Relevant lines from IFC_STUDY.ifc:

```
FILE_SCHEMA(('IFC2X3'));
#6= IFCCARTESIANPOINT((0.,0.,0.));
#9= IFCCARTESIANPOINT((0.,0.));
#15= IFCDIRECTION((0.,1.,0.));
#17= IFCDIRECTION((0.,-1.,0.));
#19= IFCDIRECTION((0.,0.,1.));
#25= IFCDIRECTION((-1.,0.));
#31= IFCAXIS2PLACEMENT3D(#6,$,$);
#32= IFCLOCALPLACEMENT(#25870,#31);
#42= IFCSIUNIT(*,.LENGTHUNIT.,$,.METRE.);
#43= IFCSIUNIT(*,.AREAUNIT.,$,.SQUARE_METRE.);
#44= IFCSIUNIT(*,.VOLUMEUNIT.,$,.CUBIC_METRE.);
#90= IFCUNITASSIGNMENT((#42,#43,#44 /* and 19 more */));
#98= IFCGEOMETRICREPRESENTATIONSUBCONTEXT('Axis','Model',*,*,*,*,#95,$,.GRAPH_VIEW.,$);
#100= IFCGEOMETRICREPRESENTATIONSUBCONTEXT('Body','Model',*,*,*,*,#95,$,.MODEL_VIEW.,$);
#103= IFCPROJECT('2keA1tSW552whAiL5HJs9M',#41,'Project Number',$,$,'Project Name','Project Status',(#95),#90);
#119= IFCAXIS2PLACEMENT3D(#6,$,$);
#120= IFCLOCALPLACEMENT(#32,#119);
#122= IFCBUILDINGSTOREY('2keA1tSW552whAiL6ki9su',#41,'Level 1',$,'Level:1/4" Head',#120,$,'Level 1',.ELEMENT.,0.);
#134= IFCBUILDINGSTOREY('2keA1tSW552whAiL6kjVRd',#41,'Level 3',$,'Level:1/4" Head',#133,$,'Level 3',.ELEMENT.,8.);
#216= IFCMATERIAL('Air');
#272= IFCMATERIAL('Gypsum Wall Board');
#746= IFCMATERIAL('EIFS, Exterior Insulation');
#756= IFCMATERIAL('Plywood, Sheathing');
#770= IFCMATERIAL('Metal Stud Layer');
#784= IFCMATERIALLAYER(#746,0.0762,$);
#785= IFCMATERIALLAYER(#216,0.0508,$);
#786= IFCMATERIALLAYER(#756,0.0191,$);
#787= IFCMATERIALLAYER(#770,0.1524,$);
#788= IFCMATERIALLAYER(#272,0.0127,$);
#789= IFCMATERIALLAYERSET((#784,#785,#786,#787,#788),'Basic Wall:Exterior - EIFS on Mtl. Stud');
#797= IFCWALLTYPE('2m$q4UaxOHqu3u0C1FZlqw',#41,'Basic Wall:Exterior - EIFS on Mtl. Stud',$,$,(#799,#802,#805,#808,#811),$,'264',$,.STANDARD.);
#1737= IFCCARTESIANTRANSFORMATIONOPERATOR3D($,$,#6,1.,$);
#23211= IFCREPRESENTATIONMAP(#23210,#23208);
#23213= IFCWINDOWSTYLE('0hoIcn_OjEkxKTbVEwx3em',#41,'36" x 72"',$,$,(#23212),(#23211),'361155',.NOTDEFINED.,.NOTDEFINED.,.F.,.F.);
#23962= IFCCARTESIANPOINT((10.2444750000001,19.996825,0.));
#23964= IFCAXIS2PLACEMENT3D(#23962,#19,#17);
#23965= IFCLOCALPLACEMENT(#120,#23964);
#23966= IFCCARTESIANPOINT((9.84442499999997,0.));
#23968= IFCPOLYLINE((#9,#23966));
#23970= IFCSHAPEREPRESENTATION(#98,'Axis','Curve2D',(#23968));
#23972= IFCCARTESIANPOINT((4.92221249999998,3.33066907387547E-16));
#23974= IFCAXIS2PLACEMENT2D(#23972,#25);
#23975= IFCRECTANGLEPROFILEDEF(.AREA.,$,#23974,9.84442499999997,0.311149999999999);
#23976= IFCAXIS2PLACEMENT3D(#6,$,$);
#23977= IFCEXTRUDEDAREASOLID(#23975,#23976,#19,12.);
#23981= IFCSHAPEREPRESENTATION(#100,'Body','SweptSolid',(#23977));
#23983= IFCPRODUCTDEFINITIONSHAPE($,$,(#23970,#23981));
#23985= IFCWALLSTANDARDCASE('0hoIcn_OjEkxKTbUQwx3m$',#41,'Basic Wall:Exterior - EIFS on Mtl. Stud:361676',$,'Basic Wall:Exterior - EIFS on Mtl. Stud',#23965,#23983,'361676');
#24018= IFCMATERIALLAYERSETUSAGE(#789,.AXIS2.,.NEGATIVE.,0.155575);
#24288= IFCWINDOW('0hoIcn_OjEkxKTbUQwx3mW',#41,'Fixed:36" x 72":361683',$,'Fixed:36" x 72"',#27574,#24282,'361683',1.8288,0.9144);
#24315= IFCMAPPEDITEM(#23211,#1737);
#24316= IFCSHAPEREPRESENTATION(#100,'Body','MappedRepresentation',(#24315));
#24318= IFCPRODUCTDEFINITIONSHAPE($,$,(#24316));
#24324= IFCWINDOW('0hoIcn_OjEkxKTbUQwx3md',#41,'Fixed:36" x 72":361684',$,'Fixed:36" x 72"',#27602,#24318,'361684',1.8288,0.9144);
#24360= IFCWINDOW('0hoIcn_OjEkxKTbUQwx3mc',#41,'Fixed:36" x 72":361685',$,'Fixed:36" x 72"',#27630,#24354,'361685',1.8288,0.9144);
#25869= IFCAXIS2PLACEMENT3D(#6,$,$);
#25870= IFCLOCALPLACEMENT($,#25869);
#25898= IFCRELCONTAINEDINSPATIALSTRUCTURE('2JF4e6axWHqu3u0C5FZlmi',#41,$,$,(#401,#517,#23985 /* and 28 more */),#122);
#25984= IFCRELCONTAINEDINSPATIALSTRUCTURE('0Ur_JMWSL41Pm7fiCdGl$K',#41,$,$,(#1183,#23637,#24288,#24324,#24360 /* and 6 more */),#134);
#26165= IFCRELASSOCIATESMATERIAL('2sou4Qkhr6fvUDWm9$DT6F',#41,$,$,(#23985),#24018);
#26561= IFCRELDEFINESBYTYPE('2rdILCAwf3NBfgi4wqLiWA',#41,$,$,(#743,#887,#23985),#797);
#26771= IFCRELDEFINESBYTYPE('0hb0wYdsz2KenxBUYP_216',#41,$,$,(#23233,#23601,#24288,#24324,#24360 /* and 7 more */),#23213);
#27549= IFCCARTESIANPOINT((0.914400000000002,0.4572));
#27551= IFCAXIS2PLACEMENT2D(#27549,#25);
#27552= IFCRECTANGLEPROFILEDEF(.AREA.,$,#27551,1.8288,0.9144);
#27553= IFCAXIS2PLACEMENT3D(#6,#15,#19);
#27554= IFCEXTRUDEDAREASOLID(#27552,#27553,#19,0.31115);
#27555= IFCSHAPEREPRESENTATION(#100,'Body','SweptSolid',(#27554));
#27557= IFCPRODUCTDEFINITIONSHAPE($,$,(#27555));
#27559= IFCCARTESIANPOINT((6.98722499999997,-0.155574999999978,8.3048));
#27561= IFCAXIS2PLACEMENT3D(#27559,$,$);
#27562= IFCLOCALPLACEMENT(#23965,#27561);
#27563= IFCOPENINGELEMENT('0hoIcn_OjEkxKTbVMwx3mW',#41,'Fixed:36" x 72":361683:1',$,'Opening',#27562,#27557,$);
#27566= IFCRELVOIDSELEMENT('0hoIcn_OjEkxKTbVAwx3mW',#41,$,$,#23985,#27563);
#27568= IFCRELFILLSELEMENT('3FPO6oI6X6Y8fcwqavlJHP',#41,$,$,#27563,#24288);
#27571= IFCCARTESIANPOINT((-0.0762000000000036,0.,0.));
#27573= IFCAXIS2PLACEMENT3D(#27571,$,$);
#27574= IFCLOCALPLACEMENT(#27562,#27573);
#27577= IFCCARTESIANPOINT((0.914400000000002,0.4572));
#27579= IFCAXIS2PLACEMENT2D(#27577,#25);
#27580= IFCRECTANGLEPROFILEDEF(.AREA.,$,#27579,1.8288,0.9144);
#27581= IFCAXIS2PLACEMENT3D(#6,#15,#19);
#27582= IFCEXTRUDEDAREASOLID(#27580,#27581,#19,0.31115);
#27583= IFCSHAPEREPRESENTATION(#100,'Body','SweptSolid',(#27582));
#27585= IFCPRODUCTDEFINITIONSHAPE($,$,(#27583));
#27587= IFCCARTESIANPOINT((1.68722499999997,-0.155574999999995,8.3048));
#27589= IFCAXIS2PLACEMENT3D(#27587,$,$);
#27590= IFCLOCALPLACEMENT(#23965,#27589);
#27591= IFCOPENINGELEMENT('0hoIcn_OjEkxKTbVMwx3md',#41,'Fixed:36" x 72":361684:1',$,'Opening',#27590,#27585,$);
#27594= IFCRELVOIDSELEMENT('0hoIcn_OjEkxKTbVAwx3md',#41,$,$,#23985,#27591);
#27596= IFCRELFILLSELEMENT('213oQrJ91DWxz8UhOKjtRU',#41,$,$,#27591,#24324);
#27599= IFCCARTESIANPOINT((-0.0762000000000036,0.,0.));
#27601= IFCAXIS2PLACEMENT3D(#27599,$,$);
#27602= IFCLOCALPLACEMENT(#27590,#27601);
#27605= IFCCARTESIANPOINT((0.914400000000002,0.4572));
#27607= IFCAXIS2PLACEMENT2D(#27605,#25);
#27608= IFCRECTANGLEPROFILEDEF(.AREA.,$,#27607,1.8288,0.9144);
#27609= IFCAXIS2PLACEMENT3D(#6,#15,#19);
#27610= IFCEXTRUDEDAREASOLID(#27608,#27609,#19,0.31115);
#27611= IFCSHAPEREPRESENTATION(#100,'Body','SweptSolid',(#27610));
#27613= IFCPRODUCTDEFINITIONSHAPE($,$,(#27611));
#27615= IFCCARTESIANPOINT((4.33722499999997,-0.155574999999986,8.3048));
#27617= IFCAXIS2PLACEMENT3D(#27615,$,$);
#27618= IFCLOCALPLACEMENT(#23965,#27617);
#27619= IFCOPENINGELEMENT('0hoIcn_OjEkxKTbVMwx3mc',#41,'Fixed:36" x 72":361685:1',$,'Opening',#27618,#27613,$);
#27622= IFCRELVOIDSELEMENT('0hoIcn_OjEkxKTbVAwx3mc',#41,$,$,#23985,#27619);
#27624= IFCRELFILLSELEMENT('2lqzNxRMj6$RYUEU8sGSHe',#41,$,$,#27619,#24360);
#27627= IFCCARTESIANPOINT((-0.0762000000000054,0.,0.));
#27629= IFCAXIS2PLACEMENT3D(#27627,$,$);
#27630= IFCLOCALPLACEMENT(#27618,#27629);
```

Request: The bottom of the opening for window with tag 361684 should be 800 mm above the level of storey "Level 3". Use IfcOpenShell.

```python
import numpy as np
import ifcopenshell
import ifcopenshell.api.geometry
import ifcopenshell.geom
import ifcopenshell.util.element
import ifcopenshell.util.placement
import ifcopenshell.util.shape
import ifcopenshell.util.unit

model = ifcopenshell.open("IFC_STUDY.ifc")
unit_scale = ifcopenshell.util.unit.calculate_unit_scale(model)

window = model.by_guid("0hoIcn_OjEkxKTbUQwx3md")
opening = window.FillsVoids[0].RelatingOpeningElement
storey = ifcopenshell.util.element.get_container(window, ifc_class="IfcBuildingStorey")
level = ifcopenshell.util.placement.get_local_placement(storey.ObjectPlacement)[2, 3]

# The opening's origin need not be at the sill, so measure its lowest point.
shape = ifcopenshell.geom.create_shape(ifcopenshell.geom.settings(), opening)
bottom = ifcopenshell.util.shape.get_shape_bottom_elevation(shape, shape.geometry) / unit_scale
dz = level + 0.8 / unit_scale - bottom

shift = np.array([0.0, 0.0, dz])
# The window is placed relative to its opening, so it follows when the opening moves.
matrix = ifcopenshell.util.placement.get_local_placement(opening.ObjectPlacement)
matrix[:3, 3] += shift
ifcopenshell.api.geometry.edit_object_placement(
    model, product=opening, matrix=matrix, is_si=False, should_transform_children=True
)

print(f"moved by {dz * unit_scale:+.3f} m")

model.write("IFC_STUDY_v2.ifc")
```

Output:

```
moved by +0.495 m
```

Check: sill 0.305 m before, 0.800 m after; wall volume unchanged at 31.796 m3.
